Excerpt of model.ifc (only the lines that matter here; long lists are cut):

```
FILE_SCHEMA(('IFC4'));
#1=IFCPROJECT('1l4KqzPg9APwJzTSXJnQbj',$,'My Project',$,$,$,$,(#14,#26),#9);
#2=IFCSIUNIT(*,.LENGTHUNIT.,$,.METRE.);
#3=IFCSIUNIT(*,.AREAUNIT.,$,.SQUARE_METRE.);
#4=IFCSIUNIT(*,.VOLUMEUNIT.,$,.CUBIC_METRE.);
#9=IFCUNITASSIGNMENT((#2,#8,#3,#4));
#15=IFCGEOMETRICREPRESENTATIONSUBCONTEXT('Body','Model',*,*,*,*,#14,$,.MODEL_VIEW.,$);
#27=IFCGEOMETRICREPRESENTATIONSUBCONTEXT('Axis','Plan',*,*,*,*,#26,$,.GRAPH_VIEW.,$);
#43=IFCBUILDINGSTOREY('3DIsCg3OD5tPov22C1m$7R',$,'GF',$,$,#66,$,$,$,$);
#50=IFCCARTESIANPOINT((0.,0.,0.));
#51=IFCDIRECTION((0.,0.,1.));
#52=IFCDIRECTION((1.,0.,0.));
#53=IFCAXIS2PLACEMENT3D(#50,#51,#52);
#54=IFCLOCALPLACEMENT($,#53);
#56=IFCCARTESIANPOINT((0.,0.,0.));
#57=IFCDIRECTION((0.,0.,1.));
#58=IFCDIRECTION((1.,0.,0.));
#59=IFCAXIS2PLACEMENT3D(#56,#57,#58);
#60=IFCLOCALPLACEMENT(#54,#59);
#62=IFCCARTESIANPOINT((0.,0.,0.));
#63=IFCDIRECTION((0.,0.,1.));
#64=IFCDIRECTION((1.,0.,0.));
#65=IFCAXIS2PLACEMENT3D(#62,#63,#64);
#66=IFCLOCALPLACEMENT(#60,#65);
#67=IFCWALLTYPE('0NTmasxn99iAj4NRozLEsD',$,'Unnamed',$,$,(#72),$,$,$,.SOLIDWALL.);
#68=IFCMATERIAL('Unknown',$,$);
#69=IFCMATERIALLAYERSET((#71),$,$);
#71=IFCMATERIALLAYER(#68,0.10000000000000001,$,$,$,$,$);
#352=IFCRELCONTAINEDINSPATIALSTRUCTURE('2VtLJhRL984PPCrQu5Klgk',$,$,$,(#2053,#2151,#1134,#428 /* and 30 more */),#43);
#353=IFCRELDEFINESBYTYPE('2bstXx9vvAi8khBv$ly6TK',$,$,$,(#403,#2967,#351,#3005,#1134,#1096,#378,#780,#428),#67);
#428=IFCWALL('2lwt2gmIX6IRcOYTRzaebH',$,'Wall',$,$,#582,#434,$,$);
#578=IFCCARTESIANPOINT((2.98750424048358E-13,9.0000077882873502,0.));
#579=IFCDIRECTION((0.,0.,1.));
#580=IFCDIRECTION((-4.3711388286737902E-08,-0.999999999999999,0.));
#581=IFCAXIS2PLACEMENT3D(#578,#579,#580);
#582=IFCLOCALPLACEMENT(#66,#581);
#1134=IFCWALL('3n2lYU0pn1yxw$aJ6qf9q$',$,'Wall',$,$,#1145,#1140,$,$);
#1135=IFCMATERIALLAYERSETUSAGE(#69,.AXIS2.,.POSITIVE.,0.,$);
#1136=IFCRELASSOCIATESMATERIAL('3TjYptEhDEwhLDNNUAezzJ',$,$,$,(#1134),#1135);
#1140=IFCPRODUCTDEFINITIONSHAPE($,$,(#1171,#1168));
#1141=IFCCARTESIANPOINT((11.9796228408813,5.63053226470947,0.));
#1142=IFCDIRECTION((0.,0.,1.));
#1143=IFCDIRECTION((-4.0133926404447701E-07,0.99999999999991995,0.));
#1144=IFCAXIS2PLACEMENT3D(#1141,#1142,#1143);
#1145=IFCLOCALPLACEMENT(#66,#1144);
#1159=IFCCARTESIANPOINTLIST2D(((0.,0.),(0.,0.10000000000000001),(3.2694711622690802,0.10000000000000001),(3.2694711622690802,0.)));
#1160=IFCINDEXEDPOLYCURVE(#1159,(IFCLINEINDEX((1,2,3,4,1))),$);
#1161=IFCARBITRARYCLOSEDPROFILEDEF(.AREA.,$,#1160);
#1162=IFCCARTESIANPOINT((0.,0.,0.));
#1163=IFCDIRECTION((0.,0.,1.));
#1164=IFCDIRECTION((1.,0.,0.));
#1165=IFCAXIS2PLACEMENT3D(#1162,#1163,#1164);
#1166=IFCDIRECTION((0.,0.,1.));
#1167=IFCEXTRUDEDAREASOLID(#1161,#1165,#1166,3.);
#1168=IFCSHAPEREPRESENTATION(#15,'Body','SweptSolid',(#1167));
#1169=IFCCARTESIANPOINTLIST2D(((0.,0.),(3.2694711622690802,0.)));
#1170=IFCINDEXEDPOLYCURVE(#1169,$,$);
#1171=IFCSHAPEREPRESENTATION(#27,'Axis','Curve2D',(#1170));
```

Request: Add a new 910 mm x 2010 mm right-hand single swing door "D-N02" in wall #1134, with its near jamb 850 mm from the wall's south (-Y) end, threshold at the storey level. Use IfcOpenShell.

```python
import numpy as np
import ifcopenshell
import ifcopenshell.api.feature
import ifcopenshell.api.geometry
import ifcopenshell.api.root
import ifcopenshell.api.spatial
import ifcopenshell.geom
import ifcopenshell.util.element
import ifcopenshell.util.placement
import ifcopenshell.util.representation
import ifcopenshell.util.shape
import ifcopenshell.util.unit

model = ifcopenshell.open("model.ifc")
unit_scale = ifcopenshell.util.unit.calculate_unit_scale(model)
settings = ifcopenshell.geom.settings()


def volume(element):
    """Net volume in cubic metres, openings subtracted."""
    shape = ifcopenshell.geom.create_shape(settings, element)
    return ifcopenshell.util.shape.get_volume(shape.geometry)


wall = model.by_guid("3n2lYU0pn1yxw$aJ6qf9q$")
storey = ifcopenshell.util.element.get_container(wall, ifc_class="IfcBuildingStorey")
context = ifcopenshell.util.representation.get_context(model, "Model", "Body", "MODEL_VIEW")
before = volume(wall)

width, height, from_end, sill = 0.91, 2.01, 0.85, 0.0  # metres

# The wall runs along its own X axis, and the end named is its -X end.
wall_shape = ifcopenshell.geom.create_shape(settings, wall)
x, y, z = ifcopenshell.util.shape.get_vertices(wall_shape.geometry).T
start = x.min() + from_end
face, thickness = float(y.min()), float(y.max() - y.min())
wall_matrix = ifcopenshell.util.placement.get_local_placement(wall.ObjectPlacement)
level = ifcopenshell.util.placement.get_local_placement(storey.ObjectPlacement)[2, 3]


def in_wall(x, y):
    """Placement at x, y metres in the wall's axes, at sill height."""
    matrix = wall_matrix.copy()
    matrix[:, 3] = wall_matrix @ np.array([x / unit_scale, y / unit_scale, 0.0, 1.0])
    matrix[2, 3] = level + sill / unit_scale
    return matrix


# Opening: a box that overshoots both wall faces by 50 mm.
opening = ifcopenshell.api.root.create_entity(model, ifc_class="IfcOpeningElement", predefined_type="OPENING")
box = ifcopenshell.api.geometry.add_wall_representation(
    model, context=context, length=width, height=height, thickness=thickness + 0.1
)
ifcopenshell.api.geometry.assign_representation(model, product=opening, representation=box)
ifcopenshell.api.geometry.edit_object_placement(model, product=opening, matrix=in_wall(start, face - 0.05), is_si=False)
ifcopenshell.api.feature.add_feature(model, feature=opening, element=wall)

door = ifcopenshell.api.root.create_entity(model, ifc_class="IfcDoor", name="D-N02", predefined_type="DOOR")
door.OverallWidth, door.OverallHeight = width / unit_scale, height / unit_scale
door.OperationType = "SINGLE_SWING_RIGHT"
body = ifcopenshell.api.geometry.add_door_representation(
    model,
    context=context,
    overall_width=door.OverallWidth,
    overall_height=door.OverallHeight,
    operation_type="SINGLE_SWING_RIGHT",
    lining_properties={"LiningDepth": thickness / unit_scale, "ThresholdDepth": thickness / unit_scale},
)
ifcopenshell.api.geometry.assign_representation(model, product=door, representation=body)
ifcopenshell.api.spatial.assign_container(model, products=[door], relating_structure=storey)
ifcopenshell.api.feature.add_filling(model, opening=opening, element=door)

# The lining spans the wall, so the door starts at the wall face.
ifcopenshell.api.geometry.edit_object_placement(model, product=door, matrix=in_wall(start, face), is_si=False)

after = volume(wall)

print(f"wall volume {before:.3f} -> {after:.3f} m3")

model.write("model_rev.ifc")
```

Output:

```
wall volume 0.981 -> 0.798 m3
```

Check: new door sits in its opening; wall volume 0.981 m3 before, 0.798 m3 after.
